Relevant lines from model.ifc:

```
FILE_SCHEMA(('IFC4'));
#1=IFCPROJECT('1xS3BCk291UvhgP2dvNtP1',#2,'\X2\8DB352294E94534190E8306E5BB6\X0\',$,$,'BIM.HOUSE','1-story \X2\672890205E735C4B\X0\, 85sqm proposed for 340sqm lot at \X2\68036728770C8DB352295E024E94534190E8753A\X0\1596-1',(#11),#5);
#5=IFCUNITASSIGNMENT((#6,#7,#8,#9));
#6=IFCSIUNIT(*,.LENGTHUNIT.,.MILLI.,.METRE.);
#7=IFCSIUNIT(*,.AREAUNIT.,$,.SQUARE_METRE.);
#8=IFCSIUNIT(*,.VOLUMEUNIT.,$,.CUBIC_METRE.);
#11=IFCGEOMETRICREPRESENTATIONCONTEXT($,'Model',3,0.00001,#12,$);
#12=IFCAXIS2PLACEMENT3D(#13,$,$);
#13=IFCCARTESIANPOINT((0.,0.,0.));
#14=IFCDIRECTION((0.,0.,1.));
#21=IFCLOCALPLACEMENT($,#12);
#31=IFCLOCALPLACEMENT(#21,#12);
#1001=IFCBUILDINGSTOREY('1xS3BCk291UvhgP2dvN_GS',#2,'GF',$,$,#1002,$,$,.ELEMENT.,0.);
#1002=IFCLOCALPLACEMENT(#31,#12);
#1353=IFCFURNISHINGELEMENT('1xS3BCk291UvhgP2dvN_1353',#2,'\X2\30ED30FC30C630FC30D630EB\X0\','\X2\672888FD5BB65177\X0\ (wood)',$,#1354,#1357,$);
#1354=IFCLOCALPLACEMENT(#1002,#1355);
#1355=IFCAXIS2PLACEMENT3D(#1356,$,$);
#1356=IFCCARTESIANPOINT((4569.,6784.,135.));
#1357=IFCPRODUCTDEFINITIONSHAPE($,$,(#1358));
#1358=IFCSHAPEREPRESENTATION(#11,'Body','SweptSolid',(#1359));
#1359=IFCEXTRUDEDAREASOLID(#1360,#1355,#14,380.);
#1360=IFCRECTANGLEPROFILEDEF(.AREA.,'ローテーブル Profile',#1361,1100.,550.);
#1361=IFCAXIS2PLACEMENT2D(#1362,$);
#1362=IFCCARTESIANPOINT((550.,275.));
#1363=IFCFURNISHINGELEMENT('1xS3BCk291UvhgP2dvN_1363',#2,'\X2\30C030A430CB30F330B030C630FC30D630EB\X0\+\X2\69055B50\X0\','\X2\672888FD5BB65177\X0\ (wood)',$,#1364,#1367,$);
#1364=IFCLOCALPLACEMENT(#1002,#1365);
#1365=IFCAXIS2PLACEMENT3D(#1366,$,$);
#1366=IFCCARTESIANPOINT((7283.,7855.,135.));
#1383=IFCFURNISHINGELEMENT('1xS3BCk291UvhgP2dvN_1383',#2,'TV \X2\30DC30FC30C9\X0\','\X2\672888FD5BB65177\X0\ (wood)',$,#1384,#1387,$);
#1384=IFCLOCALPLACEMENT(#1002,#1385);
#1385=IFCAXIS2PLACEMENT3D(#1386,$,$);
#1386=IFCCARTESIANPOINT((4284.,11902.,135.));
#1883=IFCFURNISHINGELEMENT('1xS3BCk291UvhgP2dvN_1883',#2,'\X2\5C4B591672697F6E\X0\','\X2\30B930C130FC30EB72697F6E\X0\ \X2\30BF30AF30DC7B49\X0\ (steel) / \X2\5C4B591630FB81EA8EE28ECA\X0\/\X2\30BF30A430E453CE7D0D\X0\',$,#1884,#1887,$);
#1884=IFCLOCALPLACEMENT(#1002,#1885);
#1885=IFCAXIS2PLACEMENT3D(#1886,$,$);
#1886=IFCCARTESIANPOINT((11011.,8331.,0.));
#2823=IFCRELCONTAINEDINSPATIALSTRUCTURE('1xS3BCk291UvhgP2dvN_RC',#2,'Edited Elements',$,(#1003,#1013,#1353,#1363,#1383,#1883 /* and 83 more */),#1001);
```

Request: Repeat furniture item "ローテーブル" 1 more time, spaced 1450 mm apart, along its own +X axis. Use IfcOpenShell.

```python
import ifcopenshell
import ifcopenshell.api.geometry
import ifcopenshell.api.root
import ifcopenshell.util.element
import ifcopenshell.util.placement

model = ifcopenshell.open("model.ifc")


def reuse_history(source, copy):
    """copy_class also copies each property set's owner history, people and application; keep the originals."""
    for rel in copy.IsDefinedBy:
        if rel.is_a("IfcRelDefinesByProperties") and (history := rel.RelatingPropertyDefinition.OwnerHistory):
            rel.RelatingPropertyDefinition.OwnerHistory = source.OwnerHistory
            ifcopenshell.util.element.remove_deep2(model, history)


source = model.by_id(1353)
base = ifcopenshell.util.placement.get_local_placement(source.ObjectPlacement)
step = base[:3, 0] * 1450.0

for i in range(1, 2):
    copy = ifcopenshell.api.root.copy_class(model, product=source)
    copy.Representation = ifcopenshell.util.element.copy_deep(
        model, source.Representation, exclude=["IfcGeometricRepresentationContext", "IfcRepresentationMap"]
    )
    reuse_history(source, copy)
    matrix = base.copy()
    matrix[:3, 3] += i * step
    print("added at", matrix[:3, 3].round(3) + 0.0)
    ifcopenshell.api.geometry.edit_object_placement(model, product=copy, matrix=matrix, is_si=False)

model.write("model-out.ifc")
```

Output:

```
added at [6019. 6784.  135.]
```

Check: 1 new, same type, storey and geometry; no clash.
